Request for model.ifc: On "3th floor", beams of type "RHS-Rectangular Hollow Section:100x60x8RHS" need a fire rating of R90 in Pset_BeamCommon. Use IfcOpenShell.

First a look at what the model holds.

```python
import ifcopenshell
import ifcopenshell.util.element

model = ifcopenshell.open("model.ifc")
print(model.schema)
storey = next(s for s in model.by_type("IfcBuildingStorey") if s.Name == "3th floor")
beams = [e for e in ifcopenshell.util.element.get_decomposition(storey) if e.is_a("IfcBeam")]
seen = {}
for e in beams:
    element_type = ifcopenshell.util.element.get_type(e)
    key = (element_type.Name if element_type != e and element_type else None, ifcopenshell.util.element.get_pset(e, "Pset_BeamCommon", "FireRating"))
    seen[key] = seen.get(key, 0) + 1
for (name, value), count in sorted(seen.items(), key=str):
    print(count, "x", name, "|", value)
```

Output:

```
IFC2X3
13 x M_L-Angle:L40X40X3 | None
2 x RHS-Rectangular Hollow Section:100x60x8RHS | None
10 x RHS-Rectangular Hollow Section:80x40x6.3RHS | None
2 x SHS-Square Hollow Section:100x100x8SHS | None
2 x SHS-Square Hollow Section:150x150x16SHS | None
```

```python
import ifcopenshell
import ifcopenshell.api.pset
import ifcopenshell.util.element

model = ifcopenshell.open("model.ifc")

storey = next(s for s in model.by_type("IfcBuildingStorey") if s.Name == "3th floor")
beams = [e for e in ifcopenshell.util.element.get_decomposition(storey) if e.is_a("IfcBeam")]

count = 0
for e in beams:
    element_type = ifcopenshell.util.element.get_type(e)
    if element_type in (None, e) or element_type.Name != "RHS-Rectangular Hollow Section:100x60x8RHS":
        continue
    # add_pset returns the element's existing set when there is one.
    pset = ifcopenshell.api.pset.add_pset(model, product=e, name="Pset_BeamCommon")
    ifcopenshell.api.pset.edit_pset(model, pset=pset, properties={"FireRating": "R90"})
    count += 1

print(count, "beams updated")

model.write("model-out.ifc")
```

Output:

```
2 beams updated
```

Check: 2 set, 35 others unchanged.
